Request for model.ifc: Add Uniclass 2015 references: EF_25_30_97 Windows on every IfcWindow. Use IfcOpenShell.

First a look at what the model holds.

```python
import ifcopenshell

model = ifcopenshell.open("model.ifc")
print(model.schema)
print("classifications:", [c.Name for c in model.by_type("IfcClassification")])
for ifc_class in ("IfcDoor", "IfcRoof", "IfcStair", "IfcWall", "IfcWindow"):
    print(ifc_class, len(model.by_type(ifc_class)))
```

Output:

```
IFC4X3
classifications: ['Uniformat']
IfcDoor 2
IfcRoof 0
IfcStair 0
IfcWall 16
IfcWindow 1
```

```python
import ifcopenshell
import ifcopenshell.api.classification

model = ifcopenshell.open("model.ifc")

system = ifcopenshell.api.classification.add_classification(model, classification="Uniclass 2015")

codes = {
    "IfcWindow": ("EF_25_30_97", "Windows"),
}
for ifc_class, (code, name) in codes.items():
    products = model.by_type(ifc_class)
    ifcopenshell.api.classification.add_reference(
        model, products=products, classification=system, identification=code, name=name
    )
    print(code, len(products))

model.write("model_v2.ifc")
```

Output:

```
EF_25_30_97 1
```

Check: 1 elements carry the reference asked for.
